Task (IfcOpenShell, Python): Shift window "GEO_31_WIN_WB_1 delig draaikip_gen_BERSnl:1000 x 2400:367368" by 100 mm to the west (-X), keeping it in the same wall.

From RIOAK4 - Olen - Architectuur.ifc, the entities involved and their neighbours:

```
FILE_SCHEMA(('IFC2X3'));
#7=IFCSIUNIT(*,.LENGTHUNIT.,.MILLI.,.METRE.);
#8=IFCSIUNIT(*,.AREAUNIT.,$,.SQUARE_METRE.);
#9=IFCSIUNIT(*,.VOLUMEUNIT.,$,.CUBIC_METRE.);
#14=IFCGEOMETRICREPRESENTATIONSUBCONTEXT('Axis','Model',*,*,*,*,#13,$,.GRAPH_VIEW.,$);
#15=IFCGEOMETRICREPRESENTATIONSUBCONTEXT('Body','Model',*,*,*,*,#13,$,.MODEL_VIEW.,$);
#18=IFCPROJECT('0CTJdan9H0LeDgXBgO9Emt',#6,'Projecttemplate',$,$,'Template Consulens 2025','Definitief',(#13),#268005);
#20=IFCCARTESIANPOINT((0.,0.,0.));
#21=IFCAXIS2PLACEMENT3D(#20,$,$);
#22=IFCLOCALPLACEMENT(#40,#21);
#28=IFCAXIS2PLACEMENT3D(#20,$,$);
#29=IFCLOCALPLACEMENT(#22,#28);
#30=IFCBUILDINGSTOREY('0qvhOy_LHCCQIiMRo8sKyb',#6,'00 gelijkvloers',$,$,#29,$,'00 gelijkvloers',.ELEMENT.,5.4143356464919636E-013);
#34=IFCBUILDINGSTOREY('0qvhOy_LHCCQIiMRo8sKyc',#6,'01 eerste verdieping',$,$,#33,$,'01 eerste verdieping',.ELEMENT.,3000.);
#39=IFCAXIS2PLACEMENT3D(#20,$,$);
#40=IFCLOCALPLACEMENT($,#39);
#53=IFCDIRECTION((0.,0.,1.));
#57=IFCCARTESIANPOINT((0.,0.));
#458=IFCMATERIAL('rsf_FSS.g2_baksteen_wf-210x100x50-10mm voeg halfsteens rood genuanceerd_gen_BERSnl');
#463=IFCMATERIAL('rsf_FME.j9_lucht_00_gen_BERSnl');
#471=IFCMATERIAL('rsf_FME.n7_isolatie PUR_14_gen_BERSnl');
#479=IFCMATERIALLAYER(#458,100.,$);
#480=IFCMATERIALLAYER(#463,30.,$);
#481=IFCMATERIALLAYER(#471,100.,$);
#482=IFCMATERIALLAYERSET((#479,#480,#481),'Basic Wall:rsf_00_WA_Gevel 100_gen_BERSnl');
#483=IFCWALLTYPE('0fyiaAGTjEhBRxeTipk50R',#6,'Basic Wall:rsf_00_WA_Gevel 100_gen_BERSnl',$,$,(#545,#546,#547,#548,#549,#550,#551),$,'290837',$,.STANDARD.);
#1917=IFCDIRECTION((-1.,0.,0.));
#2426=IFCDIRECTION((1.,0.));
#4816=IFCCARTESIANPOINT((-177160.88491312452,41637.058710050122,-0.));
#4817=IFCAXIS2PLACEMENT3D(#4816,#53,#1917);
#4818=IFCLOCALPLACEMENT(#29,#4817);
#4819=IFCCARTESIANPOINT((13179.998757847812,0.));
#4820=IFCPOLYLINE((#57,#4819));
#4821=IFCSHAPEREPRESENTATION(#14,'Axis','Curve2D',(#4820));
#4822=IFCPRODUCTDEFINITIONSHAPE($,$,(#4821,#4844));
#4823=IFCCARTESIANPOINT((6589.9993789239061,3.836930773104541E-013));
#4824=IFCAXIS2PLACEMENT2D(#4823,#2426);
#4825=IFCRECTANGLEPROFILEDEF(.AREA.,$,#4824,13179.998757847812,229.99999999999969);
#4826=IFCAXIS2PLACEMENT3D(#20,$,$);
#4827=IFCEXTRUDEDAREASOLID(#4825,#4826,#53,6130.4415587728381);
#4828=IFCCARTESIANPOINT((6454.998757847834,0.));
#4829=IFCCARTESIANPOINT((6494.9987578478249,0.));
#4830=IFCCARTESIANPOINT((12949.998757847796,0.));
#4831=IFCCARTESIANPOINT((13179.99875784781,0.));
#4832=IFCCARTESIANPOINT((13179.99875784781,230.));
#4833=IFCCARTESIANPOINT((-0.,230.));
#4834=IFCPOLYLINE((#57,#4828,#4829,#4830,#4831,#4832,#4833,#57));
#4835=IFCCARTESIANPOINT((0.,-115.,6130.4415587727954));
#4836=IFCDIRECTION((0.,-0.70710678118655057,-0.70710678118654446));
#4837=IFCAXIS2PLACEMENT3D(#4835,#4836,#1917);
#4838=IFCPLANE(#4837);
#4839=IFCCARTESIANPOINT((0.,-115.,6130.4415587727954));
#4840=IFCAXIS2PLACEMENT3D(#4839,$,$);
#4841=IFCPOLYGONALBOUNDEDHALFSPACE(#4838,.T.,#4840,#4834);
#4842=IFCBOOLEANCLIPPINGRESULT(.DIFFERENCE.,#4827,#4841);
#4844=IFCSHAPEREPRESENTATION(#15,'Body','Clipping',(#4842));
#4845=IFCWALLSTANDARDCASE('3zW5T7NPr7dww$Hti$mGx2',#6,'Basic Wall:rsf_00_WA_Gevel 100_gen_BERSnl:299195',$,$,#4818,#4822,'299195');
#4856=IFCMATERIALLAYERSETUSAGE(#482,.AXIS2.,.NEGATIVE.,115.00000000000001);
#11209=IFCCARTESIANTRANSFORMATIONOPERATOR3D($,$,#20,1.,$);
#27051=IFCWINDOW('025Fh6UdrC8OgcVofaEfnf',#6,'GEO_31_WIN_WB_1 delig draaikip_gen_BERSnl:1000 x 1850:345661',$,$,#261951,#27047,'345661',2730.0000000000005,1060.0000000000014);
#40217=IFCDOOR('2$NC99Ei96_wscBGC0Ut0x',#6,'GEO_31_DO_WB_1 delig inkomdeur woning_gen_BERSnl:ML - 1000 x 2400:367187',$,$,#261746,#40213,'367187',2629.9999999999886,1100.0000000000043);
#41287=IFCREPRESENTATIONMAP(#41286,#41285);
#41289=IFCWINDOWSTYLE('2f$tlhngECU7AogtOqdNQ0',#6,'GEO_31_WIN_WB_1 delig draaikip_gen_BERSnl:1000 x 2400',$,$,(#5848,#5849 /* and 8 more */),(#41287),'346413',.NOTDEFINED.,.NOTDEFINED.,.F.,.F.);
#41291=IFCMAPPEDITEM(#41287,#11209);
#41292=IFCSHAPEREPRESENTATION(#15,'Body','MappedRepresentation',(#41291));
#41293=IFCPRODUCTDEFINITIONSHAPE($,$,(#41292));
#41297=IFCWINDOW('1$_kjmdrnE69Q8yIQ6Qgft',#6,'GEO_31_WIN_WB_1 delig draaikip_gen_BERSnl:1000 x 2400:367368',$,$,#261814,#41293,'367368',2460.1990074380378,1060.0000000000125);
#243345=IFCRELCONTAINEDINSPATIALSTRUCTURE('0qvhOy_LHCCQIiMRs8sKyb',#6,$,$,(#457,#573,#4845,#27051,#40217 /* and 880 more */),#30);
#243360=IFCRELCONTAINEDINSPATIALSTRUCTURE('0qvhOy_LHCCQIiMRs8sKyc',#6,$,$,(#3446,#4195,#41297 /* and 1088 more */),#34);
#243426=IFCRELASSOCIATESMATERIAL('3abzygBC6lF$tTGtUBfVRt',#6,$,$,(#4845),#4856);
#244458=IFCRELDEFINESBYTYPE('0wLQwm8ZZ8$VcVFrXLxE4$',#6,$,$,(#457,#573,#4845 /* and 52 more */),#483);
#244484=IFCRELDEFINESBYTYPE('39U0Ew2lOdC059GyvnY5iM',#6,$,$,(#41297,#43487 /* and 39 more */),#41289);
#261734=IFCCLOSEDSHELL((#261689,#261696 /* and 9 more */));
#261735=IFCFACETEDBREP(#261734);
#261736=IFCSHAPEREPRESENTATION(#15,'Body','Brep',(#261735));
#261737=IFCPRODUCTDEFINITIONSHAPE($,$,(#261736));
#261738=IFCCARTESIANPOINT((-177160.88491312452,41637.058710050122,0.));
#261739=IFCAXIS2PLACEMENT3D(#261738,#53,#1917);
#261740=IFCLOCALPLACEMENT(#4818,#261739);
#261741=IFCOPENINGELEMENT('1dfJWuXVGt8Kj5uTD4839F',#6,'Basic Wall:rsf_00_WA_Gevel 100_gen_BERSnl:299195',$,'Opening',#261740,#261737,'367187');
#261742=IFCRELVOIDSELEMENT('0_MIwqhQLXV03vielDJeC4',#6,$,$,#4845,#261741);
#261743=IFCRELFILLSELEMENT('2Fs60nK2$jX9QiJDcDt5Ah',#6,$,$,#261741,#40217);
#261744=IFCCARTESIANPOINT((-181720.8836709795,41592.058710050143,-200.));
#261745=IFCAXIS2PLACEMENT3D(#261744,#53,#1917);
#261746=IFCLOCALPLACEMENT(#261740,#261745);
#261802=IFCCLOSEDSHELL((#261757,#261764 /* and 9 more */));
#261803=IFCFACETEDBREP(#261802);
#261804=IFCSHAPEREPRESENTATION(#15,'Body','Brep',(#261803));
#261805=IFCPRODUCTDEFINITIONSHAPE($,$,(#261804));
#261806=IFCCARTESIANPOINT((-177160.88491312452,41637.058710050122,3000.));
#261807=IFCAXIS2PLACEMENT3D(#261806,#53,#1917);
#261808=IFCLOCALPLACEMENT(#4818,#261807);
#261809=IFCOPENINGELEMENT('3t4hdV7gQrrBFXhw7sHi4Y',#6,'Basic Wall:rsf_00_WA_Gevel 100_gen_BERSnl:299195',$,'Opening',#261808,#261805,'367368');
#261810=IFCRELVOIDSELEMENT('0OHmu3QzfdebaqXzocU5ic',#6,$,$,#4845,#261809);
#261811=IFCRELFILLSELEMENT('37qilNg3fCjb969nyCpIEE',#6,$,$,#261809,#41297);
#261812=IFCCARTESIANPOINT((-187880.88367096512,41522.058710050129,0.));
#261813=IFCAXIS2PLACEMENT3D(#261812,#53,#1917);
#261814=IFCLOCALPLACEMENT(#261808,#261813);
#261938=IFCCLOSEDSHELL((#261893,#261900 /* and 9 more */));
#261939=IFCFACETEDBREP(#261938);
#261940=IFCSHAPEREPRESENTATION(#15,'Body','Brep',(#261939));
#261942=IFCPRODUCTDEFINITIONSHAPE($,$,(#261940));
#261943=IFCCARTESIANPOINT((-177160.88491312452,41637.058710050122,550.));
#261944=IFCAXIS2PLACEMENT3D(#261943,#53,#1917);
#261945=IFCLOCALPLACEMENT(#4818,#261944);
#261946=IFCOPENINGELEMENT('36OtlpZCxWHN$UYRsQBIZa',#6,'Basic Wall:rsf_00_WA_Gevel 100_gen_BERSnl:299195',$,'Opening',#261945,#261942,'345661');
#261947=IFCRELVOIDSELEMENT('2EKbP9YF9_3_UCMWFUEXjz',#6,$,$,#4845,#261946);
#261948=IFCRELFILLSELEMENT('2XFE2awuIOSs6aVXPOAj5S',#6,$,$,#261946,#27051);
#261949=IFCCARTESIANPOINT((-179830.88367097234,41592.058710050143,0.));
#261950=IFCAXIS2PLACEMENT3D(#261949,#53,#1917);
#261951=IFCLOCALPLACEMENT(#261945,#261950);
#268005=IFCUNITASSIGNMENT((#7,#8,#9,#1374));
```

```python
import ifcopenshell
import ifcopenshell.api.geometry
import ifcopenshell.util.placement
import ifcopenshell.util.unit

model = ifcopenshell.open("RIOAK4 - Olen - Architectuur.ifc")
unit_scale = ifcopenshell.util.unit.calculate_unit_scale(model)

window = model.by_id(41297)
opening = window.FillsVoids[0].RelatingOpeningElement
wall = opening.VoidsElements[0].RelatingBuildingElement

wall_matrix = ifcopenshell.util.placement.get_local_placement(wall.ObjectPlacement)
shift = wall_matrix[:3, 0] * 0.1 / unit_scale
before = ifcopenshell.util.placement.get_local_placement(window.ObjectPlacement)[:3, 3].copy()

# The window is placed relative to its opening, so it follows when the opening moves.
matrix = ifcopenshell.util.placement.get_local_placement(opening.ObjectPlacement)
matrix[:3, 3] += shift
ifcopenshell.api.geometry.edit_object_placement(
    model, product=opening, matrix=matrix, is_si=False, should_transform_children=True
)

after = ifcopenshell.util.placement.get_local_placement(window.ObjectPlacement)[:3, 3]
print("window moved by", (after - before).round(3) + 0.0)

model.write("RIOAK4 - Olen - Architectuur_updated.ifc")
```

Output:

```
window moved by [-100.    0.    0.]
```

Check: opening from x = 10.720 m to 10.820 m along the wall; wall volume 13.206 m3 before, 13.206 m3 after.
